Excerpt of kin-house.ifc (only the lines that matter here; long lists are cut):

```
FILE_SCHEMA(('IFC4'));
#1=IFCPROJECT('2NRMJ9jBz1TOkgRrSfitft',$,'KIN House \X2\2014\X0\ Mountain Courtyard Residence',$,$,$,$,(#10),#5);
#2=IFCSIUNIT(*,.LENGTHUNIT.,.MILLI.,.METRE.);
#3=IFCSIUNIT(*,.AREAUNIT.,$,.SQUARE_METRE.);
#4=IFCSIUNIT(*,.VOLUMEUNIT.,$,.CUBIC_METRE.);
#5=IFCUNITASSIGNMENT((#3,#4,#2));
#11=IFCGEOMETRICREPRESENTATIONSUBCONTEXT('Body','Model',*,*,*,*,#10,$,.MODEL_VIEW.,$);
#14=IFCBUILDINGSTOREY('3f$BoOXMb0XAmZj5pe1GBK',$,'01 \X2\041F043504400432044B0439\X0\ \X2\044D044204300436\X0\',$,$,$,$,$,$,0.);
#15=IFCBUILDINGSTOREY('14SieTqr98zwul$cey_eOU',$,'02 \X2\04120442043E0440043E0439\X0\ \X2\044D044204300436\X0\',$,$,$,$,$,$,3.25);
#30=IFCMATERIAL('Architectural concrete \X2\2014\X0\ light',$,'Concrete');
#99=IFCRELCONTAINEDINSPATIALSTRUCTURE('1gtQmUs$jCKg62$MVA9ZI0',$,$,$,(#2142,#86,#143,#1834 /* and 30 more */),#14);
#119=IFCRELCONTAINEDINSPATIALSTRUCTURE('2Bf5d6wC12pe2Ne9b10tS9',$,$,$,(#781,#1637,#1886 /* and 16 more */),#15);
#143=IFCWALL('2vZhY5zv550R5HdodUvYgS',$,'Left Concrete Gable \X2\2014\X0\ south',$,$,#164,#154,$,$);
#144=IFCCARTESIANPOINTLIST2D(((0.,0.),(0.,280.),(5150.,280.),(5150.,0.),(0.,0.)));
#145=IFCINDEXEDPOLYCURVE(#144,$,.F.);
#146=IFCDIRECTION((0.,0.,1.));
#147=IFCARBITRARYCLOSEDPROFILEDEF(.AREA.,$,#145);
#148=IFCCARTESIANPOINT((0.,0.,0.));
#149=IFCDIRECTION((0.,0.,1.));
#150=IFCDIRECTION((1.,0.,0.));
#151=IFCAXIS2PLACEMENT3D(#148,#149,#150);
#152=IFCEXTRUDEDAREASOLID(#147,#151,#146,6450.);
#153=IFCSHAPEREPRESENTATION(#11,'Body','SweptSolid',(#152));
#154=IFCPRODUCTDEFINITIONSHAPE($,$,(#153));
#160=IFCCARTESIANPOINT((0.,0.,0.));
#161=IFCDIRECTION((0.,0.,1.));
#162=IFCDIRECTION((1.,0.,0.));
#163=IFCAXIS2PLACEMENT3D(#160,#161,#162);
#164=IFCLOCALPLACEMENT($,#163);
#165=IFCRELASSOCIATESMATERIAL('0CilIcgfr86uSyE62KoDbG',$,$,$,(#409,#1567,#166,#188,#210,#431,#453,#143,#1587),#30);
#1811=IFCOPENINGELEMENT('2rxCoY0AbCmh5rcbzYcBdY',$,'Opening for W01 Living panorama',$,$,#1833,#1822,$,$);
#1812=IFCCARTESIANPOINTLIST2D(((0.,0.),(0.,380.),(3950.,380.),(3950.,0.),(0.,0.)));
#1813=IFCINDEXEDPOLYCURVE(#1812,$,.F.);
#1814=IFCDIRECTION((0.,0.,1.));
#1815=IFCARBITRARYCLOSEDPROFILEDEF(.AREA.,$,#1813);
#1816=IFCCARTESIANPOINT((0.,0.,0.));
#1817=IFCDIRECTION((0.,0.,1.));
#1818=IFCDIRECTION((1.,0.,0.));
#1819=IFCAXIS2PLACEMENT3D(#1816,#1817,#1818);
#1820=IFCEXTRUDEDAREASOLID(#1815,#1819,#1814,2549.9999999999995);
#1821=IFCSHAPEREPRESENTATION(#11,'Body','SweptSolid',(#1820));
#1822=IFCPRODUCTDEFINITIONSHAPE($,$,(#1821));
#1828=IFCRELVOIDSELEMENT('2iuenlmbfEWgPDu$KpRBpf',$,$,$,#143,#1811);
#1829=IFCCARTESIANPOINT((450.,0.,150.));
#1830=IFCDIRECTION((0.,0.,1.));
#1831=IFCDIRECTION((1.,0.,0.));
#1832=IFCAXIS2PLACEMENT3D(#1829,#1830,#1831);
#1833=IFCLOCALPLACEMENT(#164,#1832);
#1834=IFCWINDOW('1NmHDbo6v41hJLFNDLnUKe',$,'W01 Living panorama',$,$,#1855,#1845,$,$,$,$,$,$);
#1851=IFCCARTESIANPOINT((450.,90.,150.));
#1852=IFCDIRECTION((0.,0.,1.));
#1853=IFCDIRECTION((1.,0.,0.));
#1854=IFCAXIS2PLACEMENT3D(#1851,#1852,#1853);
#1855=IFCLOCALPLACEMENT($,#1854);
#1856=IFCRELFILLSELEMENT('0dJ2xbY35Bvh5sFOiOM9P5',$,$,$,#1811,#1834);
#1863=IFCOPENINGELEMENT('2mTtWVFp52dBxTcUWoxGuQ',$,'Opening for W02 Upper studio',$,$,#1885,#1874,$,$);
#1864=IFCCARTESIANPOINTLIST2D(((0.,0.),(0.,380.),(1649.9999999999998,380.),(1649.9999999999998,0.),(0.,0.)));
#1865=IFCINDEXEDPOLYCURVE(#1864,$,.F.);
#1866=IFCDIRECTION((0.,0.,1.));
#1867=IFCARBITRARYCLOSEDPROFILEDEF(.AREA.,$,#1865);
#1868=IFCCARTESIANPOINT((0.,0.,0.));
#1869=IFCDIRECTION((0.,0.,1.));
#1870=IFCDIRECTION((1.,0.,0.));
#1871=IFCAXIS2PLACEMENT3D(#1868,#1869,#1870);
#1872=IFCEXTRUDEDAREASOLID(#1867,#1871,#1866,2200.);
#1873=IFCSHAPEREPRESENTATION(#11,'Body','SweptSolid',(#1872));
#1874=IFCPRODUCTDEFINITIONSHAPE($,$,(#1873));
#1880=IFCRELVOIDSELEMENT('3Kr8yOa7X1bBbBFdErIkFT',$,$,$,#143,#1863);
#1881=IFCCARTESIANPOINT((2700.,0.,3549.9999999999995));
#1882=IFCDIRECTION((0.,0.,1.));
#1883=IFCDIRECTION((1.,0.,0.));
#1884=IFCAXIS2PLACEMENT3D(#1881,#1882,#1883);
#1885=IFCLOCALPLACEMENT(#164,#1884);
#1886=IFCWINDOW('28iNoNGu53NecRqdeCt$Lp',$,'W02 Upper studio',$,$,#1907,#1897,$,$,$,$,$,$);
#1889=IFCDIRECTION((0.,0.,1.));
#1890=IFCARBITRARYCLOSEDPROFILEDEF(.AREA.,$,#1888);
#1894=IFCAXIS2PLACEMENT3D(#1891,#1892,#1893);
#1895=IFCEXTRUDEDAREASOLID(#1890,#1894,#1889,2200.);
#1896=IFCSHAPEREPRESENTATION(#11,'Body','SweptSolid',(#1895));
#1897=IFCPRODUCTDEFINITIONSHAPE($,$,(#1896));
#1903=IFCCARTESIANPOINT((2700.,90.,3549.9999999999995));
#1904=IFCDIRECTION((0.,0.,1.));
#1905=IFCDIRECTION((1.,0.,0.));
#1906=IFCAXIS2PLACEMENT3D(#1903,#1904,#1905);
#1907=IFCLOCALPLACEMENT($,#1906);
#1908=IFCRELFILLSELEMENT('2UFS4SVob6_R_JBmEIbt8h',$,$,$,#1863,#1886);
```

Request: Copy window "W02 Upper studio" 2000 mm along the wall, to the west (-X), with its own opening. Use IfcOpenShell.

```python
import ifcopenshell
import ifcopenshell.api.feature
import ifcopenshell.api.geometry
import ifcopenshell.api.root
import ifcopenshell.geom
import ifcopenshell.util.element
import ifcopenshell.util.placement
import ifcopenshell.util.shape

model = ifcopenshell.open("kin-house.ifc")
settings = ifcopenshell.geom.settings()


def volume(element):
    """Net volume in cubic metres, openings subtracted."""
    shape = ifcopenshell.geom.create_shape(settings, element)
    return ifcopenshell.util.shape.get_volume(shape.geometry)


window = model.by_guid("28iNoNGu53NecRqdeCt$Lp")
opening = window.FillsVoids[0].RelatingOpeningElement
wall = opening.VoidsElements[0].RelatingBuildingElement
before = volume(wall)
shift = ifcopenshell.util.placement.get_local_placement(wall.ObjectPlacement)[:3, 0] * -2000.0

# copy_class copies the void relationship, type, container and properties, but no geometry.
new_opening = ifcopenshell.api.root.copy_class(model, product=opening)
new_opening.Representation = ifcopenshell.util.element.copy_deep(
    model, opening.Representation, exclude=["IfcGeometricRepresentationContext", "IfcRepresentationMap"]
)
new_window = ifcopenshell.api.root.copy_class(model, product=window)
new_window.Representation = ifcopenshell.util.element.copy_deep(
    model, window.Representation, exclude=["IfcGeometricRepresentationContext", "IfcRepresentationMap"]
)
ifcopenshell.api.feature.add_filling(model, opening=new_opening, element=new_window)

for old, new in ((opening, new_opening), (window, new_window)):
    matrix = ifcopenshell.util.placement.get_local_placement(old.ObjectPlacement)
    matrix[:3, 3] += shift
    ifcopenshell.api.geometry.edit_object_placement(model, product=new, matrix=matrix, is_si=False)

after = volume(wall)

print(f"wall volume {before:.3f} -> {after:.3f} m3")

model.write("kin-house-out.ifc")
```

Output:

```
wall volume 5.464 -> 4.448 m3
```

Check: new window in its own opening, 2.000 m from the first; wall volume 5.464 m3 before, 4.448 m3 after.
